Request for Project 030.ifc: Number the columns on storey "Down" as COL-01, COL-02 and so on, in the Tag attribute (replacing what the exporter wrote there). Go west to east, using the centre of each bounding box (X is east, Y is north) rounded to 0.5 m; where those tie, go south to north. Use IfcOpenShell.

First a look at what the model holds.

```python
import ifcopenshell
import ifcopenshell.util.element
import ifcopenshell.util.placement

model = ifcopenshell.open("Project 030.ifc")
print(model.schema)
storey = next(s for s in model.by_type("IfcBuildingStorey") if s.Name == "Down")
columns = [e for e in ifcopenshell.util.element.get_decomposition(storey) if e.is_a("IfcColumn")]
for e in sorted(columns, key=lambda e: e.id()):
    origin = ifcopenshell.util.placement.get_local_placement(e.ObjectPlacement)[:3, 3]
    print(e.id(), e.Tag, e.Name, origin.round(2) + 0.0, sep=" | ")
```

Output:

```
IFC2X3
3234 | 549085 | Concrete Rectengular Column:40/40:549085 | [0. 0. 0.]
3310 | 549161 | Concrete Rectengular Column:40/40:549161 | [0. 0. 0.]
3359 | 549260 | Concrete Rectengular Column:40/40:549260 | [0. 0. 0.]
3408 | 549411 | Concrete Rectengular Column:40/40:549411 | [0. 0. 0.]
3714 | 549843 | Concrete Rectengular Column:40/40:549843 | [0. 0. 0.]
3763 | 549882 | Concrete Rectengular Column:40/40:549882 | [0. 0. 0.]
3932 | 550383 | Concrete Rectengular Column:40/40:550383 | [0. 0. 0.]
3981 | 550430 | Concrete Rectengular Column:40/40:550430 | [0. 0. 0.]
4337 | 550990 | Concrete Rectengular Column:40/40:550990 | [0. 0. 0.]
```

```python
import ifcopenshell
import ifcopenshell.geom
import ifcopenshell.util.element
import ifcopenshell.util.shape

model = ifcopenshell.open("Project 030.ifc")
settings = ifcopenshell.geom.settings()
settings.set("use-world-coords", True)


def centre(element):
    shape = ifcopenshell.geom.create_shape(settings, element)
    return ifcopenshell.util.shape.get_bbox_centroid(shape.geometry)


storey = next(s for s in model.by_type("IfcBuildingStorey") if s.Name == "Down")
columns = [e for e in ifcopenshell.util.element.get_decomposition(storey) if e.is_a("IfcColumn")]

# Insertion points can sit at a corner or the storey origin, so sort by the geometry (in metres).
centres = {e: centre(e) for e in columns}
columns.sort(key=lambda e: (round(centres[e][0] / 0.5), centres[e][1]))

for i, e in enumerate(columns, start=1):
    number = f"COL-{i:02d}"
    e.Tag = number
    print(e.id(), number)

model.write("Project 030-out.ifc")
```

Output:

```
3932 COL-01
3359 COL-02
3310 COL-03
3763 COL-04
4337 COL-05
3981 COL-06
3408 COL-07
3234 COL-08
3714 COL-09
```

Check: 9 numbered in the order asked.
